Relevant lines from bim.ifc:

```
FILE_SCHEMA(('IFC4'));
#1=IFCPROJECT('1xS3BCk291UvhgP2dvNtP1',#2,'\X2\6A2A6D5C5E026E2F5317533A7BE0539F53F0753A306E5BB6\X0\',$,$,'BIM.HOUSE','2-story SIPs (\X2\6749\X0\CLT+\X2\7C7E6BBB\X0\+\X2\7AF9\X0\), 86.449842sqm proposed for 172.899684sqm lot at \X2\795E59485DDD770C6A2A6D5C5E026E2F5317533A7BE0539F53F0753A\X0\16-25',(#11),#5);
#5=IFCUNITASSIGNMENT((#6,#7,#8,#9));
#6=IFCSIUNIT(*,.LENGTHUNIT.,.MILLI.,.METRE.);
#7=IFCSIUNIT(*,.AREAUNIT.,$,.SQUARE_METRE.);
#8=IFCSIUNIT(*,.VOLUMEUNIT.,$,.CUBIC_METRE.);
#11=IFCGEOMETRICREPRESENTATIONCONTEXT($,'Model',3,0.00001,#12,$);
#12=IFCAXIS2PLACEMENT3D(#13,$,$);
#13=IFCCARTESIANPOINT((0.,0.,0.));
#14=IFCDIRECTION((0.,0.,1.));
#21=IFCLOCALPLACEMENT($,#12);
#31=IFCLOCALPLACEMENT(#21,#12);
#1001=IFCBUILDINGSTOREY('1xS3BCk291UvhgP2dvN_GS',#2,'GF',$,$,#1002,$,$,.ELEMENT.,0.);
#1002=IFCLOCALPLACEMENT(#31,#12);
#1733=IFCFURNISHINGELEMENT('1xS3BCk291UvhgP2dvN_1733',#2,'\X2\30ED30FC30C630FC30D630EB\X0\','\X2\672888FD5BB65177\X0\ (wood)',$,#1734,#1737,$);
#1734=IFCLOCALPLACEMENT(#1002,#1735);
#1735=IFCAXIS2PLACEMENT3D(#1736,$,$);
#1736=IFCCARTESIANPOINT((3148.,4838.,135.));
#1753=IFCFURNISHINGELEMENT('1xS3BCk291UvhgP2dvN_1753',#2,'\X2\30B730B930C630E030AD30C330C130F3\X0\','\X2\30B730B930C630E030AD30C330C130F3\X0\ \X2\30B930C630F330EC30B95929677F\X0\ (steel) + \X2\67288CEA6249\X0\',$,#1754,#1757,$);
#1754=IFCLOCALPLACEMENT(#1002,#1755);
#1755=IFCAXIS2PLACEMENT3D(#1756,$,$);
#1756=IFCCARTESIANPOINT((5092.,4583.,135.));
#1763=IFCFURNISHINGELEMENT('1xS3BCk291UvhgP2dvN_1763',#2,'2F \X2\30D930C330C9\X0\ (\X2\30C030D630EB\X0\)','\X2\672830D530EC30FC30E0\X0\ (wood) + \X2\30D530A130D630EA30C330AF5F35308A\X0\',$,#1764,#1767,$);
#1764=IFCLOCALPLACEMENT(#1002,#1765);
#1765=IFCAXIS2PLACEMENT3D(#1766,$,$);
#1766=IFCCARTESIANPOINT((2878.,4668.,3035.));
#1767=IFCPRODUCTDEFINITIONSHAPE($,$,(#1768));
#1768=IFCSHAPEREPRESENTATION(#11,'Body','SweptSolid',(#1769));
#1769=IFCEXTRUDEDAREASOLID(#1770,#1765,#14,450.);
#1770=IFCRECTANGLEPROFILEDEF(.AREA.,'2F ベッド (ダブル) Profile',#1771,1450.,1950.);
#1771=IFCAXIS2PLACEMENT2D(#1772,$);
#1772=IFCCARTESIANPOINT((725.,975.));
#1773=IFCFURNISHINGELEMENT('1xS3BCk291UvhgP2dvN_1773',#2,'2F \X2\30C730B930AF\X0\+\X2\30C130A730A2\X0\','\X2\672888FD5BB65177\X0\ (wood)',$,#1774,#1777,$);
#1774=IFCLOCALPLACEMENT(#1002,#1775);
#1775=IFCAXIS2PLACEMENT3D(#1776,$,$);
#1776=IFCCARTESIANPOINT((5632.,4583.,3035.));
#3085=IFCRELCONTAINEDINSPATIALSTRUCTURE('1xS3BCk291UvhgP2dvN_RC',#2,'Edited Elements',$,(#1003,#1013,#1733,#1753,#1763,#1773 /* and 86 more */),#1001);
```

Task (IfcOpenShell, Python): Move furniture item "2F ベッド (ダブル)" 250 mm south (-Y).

```python
import ifcopenshell
import ifcopenshell.api.geometry
import ifcopenshell.util.placement
import ifcopenshell.util.unit

model = ifcopenshell.open("bim.ifc")
unit_scale = ifcopenshell.util.unit.calculate_unit_scale(model)

item = model.by_id(1763)
matrix = ifcopenshell.util.placement.get_local_placement(item.ObjectPlacement)
matrix[1, 3] -= 0.25 / unit_scale
ifcopenshell.api.geometry.edit_object_placement(model, product=item, matrix=matrix, is_si=False)

print(ifcopenshell.util.placement.get_local_placement(item.ObjectPlacement).round(3) + 0.0)

model.write("bim-out.ifc")
```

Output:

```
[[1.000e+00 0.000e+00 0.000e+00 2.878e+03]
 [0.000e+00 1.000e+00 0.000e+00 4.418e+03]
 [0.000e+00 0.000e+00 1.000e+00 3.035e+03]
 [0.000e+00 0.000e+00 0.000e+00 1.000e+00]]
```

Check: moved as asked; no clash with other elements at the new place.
